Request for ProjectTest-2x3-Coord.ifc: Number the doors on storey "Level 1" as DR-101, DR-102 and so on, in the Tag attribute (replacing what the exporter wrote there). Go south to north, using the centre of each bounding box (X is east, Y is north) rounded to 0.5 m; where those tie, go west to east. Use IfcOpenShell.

First a look at what the model holds.

```python
import ifcopenshell
import ifcopenshell.util.element
import ifcopenshell.util.placement

model = ifcopenshell.open("ProjectTest-2x3-Coord.ifc")
print(model.schema)
storey = next(s for s in model.by_type("IfcBuildingStorey") if s.Name == "Level 1")
doors = [e for e in ifcopenshell.util.element.get_decomposition(storey) if e.is_a("IfcDoor")]
for e in sorted(doors, key=lambda e: e.id()):
    origin = ifcopenshell.util.placement.get_local_placement(e.ObjectPlacement)[:3, 3]
    print(e.id(), e.Tag, e.Name, origin.round(2) + 0.0, sep=" | ")
```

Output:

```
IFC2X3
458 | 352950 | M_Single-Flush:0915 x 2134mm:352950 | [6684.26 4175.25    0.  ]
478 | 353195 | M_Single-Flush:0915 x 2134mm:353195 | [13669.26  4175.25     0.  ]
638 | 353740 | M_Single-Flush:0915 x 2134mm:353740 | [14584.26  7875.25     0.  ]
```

```python
import ifcopenshell
import ifcopenshell.geom
import ifcopenshell.util.element
import ifcopenshell.util.shape

model = ifcopenshell.open("ProjectTest-2x3-Coord.ifc")
settings = ifcopenshell.geom.settings()
settings.set("use-world-coords", True)


def centre(element):
    shape = ifcopenshell.geom.create_shape(settings, element)
    return ifcopenshell.util.shape.get_bbox_centroid(shape.geometry)


storey = next(s for s in model.by_type("IfcBuildingStorey") if s.Name == "Level 1")
doors = [e for e in ifcopenshell.util.element.get_decomposition(storey) if e.is_a("IfcDoor")]

# Insertion points can sit at a corner or the storey origin, so sort by the geometry (in metres).
centres = {e: centre(e) for e in doors}
doors.sort(key=lambda e: (round(centres[e][1] / 0.5), centres[e][0]))

for i, e in enumerate(doors, start=1):
    number = f"DR-1{i:02d}"
    e.Tag = number
    print(e.id(), number)

model.write("ProjectTest-2x3-Coord_updated.ifc")
```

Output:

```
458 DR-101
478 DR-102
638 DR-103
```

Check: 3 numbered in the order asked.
